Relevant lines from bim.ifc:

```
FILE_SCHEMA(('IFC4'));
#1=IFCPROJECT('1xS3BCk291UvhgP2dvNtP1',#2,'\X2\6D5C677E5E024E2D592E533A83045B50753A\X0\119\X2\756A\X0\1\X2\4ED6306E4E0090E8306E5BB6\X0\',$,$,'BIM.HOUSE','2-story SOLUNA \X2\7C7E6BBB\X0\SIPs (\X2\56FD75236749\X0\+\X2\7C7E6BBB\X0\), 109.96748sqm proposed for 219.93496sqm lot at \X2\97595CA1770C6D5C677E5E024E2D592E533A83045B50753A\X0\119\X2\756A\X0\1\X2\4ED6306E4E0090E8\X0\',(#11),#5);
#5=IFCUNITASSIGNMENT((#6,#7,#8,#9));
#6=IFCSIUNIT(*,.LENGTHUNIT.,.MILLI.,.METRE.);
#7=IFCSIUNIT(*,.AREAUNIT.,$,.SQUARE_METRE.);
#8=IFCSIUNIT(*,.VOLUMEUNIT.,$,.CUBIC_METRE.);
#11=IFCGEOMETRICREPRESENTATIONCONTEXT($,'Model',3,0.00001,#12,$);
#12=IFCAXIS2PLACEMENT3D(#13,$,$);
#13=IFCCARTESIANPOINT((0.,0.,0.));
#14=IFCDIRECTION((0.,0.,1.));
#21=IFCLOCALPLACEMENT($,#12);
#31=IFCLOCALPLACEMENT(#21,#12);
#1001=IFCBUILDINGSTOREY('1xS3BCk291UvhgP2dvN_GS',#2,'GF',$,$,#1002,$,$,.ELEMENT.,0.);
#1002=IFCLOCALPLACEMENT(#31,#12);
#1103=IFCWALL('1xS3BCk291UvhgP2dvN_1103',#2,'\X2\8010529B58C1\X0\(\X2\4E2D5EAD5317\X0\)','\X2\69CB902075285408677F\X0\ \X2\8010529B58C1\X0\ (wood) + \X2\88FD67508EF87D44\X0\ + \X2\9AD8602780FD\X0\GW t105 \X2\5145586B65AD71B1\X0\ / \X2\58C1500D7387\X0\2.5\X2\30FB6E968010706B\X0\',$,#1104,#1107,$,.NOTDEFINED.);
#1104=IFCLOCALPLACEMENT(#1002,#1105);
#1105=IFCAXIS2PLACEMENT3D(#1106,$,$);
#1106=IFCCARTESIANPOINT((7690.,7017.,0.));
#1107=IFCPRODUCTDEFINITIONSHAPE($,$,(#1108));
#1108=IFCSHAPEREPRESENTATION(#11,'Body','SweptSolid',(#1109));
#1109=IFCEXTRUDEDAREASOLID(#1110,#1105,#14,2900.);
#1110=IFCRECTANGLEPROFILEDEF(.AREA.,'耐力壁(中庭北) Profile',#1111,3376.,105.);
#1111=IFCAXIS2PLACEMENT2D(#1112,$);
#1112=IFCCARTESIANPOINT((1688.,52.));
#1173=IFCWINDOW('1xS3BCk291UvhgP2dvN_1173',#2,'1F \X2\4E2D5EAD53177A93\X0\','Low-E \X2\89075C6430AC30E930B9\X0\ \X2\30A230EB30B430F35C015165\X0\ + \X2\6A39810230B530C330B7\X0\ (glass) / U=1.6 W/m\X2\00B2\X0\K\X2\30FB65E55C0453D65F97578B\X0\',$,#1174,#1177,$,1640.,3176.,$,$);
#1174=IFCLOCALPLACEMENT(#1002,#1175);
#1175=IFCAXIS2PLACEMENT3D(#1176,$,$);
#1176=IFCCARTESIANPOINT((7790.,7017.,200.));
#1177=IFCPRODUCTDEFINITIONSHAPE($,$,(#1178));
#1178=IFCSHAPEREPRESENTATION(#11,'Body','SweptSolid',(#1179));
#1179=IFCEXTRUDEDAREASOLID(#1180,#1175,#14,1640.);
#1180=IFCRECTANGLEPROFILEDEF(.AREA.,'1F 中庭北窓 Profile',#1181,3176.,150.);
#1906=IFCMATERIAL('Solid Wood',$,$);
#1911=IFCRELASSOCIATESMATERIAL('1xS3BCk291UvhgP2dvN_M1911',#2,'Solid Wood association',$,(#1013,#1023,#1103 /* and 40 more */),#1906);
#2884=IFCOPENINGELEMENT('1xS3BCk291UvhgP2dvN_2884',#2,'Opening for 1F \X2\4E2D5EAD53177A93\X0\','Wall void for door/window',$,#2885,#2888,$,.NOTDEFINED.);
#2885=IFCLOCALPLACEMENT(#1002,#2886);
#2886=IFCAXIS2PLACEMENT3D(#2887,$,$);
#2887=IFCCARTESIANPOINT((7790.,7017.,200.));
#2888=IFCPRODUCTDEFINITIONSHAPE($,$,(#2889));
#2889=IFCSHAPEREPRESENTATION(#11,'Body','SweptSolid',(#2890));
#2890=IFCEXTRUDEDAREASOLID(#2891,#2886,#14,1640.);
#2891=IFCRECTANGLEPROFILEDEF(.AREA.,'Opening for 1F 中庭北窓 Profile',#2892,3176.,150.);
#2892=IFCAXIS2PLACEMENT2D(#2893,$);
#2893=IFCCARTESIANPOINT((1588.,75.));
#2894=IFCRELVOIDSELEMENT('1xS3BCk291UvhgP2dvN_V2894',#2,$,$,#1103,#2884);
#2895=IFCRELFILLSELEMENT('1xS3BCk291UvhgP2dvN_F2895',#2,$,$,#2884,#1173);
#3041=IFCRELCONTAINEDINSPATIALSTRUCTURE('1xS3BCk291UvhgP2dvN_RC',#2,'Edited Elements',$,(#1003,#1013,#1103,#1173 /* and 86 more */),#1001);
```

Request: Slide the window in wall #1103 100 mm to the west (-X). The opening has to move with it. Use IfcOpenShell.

```python
import ifcopenshell
import ifcopenshell.api.geometry
import ifcopenshell.util.placement
import ifcopenshell.util.unit

model = ifcopenshell.open("bim.ifc")
unit_scale = ifcopenshell.util.unit.calculate_unit_scale(model)

window = model.by_guid("1xS3BCk291UvhgP2dvN_1173")
opening = window.FillsVoids[0].RelatingOpeningElement
wall = opening.VoidsElements[0].RelatingBuildingElement

wall_matrix = ifcopenshell.util.placement.get_local_placement(wall.ObjectPlacement)
shift = wall_matrix[:3, 0] * -0.1 / unit_scale
before = ifcopenshell.util.placement.get_local_placement(window.ObjectPlacement)[:3, 3].copy()

# The window is not placed relative to its opening, so move both.
for product in (opening, window):
    matrix = ifcopenshell.util.placement.get_local_placement(product.ObjectPlacement)
    matrix[:3, 3] += shift
    ifcopenshell.api.geometry.edit_object_placement(model, product=product, matrix=matrix, is_si=False)

after = ifcopenshell.util.placement.get_local_placement(window.ObjectPlacement)[:3, 3]
print("window moved by", (after - before).round(3) + 0.0)

model.write("bim_updated.ifc")
```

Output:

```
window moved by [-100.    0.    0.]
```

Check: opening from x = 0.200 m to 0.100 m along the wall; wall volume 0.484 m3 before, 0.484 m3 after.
